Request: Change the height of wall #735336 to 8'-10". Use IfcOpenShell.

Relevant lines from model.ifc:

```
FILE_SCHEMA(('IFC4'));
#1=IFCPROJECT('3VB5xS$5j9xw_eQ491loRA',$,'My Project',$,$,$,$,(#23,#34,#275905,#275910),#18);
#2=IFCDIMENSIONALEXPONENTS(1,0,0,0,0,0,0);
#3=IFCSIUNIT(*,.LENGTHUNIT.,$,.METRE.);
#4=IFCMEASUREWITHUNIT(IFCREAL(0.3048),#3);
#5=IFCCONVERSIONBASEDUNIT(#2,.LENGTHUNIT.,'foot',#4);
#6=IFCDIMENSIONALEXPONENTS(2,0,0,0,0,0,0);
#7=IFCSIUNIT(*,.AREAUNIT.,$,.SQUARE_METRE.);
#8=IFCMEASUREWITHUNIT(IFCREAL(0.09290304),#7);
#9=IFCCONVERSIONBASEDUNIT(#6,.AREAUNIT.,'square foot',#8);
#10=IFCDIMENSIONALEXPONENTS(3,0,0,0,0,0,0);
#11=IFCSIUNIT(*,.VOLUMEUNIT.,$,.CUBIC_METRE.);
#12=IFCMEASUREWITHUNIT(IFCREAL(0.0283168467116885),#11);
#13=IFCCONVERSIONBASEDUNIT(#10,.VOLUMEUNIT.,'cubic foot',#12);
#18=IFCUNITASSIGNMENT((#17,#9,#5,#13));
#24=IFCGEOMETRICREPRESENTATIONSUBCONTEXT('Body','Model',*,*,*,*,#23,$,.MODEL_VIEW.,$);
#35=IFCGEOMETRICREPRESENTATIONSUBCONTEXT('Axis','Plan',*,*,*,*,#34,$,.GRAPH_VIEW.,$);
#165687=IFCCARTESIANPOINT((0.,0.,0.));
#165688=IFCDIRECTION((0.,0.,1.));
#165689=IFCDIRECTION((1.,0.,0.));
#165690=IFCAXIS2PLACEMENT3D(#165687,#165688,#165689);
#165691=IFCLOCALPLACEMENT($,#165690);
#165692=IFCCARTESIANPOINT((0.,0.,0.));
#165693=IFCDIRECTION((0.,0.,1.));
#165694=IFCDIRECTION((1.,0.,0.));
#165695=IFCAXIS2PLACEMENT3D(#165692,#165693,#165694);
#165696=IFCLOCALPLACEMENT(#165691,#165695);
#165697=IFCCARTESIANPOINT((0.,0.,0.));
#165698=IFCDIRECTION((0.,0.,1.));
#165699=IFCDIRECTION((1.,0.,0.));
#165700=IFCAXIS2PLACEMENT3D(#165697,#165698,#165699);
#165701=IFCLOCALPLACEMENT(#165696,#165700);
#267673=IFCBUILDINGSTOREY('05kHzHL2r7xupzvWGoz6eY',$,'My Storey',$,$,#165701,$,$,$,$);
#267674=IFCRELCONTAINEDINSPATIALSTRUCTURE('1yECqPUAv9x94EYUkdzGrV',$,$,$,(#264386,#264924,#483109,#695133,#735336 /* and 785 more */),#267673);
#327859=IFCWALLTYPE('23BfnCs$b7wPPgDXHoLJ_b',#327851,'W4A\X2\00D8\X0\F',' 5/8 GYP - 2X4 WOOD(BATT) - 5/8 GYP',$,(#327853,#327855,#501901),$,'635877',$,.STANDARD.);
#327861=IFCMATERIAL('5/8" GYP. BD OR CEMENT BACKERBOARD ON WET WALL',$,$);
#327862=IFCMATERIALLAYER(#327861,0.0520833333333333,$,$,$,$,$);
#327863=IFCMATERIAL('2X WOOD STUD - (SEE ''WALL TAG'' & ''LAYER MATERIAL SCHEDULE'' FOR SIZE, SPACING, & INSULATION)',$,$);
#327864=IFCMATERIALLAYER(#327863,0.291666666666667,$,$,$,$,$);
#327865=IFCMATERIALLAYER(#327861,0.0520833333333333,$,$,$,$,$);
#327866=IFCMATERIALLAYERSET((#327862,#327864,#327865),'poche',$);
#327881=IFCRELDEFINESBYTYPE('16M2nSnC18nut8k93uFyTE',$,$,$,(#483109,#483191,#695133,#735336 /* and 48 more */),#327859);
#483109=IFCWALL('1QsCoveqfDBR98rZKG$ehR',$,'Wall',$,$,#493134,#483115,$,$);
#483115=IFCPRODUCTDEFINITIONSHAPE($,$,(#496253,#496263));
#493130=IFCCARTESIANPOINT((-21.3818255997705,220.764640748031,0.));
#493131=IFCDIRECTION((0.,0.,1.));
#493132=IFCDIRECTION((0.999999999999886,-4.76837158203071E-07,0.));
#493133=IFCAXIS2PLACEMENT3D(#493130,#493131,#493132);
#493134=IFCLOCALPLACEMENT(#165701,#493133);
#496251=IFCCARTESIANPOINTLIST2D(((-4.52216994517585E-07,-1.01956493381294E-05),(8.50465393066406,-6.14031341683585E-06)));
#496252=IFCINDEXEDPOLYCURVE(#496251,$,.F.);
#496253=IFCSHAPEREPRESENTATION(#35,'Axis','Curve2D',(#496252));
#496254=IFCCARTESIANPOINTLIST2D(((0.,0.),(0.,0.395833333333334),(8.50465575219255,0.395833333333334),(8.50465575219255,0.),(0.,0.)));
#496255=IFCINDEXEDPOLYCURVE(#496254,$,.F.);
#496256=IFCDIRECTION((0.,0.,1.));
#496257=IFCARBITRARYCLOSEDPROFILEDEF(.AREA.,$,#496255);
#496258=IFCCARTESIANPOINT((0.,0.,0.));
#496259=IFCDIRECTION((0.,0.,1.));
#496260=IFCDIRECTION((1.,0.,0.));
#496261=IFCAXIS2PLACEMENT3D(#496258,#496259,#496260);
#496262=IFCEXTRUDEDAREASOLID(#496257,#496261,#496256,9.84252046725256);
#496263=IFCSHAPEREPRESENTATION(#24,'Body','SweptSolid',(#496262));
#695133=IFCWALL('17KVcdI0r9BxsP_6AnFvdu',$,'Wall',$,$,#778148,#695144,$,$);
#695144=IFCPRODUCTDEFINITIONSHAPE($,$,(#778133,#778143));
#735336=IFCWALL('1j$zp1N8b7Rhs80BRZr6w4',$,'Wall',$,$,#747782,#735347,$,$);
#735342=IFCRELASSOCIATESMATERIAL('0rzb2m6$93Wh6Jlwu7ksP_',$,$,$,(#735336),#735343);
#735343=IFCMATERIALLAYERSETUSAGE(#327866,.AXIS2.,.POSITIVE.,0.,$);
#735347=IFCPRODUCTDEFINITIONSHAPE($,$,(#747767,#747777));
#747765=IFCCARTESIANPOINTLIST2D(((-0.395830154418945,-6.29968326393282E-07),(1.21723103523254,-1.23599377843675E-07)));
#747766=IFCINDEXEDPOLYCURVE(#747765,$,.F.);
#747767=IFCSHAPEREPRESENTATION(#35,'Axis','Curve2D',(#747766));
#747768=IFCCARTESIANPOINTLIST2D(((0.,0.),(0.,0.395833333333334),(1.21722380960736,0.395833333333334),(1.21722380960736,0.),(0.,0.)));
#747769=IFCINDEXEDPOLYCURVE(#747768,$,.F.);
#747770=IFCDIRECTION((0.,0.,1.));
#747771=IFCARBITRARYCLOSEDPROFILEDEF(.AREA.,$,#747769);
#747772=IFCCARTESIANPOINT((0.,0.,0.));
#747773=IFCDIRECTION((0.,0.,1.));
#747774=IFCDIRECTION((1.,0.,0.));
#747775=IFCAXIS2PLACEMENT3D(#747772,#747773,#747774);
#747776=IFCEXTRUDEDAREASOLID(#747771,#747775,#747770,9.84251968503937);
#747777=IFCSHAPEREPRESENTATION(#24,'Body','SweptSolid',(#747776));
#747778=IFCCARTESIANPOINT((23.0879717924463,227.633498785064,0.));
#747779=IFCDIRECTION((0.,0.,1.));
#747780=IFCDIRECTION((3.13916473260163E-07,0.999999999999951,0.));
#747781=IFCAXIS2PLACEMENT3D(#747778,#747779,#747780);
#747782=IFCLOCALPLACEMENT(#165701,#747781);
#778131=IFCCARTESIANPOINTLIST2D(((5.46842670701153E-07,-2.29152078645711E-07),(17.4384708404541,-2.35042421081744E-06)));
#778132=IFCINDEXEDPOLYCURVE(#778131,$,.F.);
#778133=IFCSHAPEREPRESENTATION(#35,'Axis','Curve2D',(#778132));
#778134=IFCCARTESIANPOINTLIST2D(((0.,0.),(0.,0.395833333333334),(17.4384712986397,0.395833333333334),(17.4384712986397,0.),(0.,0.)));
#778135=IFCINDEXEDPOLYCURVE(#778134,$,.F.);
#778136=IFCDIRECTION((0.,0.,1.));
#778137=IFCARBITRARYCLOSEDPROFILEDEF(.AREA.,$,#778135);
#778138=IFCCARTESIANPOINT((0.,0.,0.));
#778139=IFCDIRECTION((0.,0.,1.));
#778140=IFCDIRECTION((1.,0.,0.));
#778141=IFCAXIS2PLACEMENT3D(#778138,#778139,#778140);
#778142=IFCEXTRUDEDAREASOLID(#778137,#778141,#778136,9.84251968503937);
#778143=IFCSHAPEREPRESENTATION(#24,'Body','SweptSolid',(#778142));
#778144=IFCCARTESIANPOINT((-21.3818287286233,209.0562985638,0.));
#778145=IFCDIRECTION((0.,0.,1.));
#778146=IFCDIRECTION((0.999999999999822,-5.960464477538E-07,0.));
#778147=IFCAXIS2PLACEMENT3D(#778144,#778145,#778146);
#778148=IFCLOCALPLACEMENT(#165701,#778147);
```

```python
import ifcopenshell
import ifcopenshell.geom
import ifcopenshell.util.representation
import ifcopenshell.util.shape
import ifcopenshell.util.unit

model = ifcopenshell.open("model.ifc")
unit_scale = ifcopenshell.util.unit.calculate_unit_scale(model)
settings = ifcopenshell.geom.settings()


def volume(element):
    """Net volume in cubic metres, openings subtracted."""
    shape = ifcopenshell.geom.create_shape(settings, element)
    return ifcopenshell.util.shape.get_volume(shape.geometry)


wall = model.by_id(735336)
before = volume(wall)

body = ifcopenshell.util.representation.get_representation(wall, "Model", "Body")
solid = body.Items[0]
old_height = solid.Depth
solid.Depth = 106 * 0.0254 / unit_scale
after = volume(wall)

print(f"height {old_height:g} -> {solid.Depth:g}, volume {before:.3f} -> {after:.3f} m3")

model.write("model_v2.ifc")
```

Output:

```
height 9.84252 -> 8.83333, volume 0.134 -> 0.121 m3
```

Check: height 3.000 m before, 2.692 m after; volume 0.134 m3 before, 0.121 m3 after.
